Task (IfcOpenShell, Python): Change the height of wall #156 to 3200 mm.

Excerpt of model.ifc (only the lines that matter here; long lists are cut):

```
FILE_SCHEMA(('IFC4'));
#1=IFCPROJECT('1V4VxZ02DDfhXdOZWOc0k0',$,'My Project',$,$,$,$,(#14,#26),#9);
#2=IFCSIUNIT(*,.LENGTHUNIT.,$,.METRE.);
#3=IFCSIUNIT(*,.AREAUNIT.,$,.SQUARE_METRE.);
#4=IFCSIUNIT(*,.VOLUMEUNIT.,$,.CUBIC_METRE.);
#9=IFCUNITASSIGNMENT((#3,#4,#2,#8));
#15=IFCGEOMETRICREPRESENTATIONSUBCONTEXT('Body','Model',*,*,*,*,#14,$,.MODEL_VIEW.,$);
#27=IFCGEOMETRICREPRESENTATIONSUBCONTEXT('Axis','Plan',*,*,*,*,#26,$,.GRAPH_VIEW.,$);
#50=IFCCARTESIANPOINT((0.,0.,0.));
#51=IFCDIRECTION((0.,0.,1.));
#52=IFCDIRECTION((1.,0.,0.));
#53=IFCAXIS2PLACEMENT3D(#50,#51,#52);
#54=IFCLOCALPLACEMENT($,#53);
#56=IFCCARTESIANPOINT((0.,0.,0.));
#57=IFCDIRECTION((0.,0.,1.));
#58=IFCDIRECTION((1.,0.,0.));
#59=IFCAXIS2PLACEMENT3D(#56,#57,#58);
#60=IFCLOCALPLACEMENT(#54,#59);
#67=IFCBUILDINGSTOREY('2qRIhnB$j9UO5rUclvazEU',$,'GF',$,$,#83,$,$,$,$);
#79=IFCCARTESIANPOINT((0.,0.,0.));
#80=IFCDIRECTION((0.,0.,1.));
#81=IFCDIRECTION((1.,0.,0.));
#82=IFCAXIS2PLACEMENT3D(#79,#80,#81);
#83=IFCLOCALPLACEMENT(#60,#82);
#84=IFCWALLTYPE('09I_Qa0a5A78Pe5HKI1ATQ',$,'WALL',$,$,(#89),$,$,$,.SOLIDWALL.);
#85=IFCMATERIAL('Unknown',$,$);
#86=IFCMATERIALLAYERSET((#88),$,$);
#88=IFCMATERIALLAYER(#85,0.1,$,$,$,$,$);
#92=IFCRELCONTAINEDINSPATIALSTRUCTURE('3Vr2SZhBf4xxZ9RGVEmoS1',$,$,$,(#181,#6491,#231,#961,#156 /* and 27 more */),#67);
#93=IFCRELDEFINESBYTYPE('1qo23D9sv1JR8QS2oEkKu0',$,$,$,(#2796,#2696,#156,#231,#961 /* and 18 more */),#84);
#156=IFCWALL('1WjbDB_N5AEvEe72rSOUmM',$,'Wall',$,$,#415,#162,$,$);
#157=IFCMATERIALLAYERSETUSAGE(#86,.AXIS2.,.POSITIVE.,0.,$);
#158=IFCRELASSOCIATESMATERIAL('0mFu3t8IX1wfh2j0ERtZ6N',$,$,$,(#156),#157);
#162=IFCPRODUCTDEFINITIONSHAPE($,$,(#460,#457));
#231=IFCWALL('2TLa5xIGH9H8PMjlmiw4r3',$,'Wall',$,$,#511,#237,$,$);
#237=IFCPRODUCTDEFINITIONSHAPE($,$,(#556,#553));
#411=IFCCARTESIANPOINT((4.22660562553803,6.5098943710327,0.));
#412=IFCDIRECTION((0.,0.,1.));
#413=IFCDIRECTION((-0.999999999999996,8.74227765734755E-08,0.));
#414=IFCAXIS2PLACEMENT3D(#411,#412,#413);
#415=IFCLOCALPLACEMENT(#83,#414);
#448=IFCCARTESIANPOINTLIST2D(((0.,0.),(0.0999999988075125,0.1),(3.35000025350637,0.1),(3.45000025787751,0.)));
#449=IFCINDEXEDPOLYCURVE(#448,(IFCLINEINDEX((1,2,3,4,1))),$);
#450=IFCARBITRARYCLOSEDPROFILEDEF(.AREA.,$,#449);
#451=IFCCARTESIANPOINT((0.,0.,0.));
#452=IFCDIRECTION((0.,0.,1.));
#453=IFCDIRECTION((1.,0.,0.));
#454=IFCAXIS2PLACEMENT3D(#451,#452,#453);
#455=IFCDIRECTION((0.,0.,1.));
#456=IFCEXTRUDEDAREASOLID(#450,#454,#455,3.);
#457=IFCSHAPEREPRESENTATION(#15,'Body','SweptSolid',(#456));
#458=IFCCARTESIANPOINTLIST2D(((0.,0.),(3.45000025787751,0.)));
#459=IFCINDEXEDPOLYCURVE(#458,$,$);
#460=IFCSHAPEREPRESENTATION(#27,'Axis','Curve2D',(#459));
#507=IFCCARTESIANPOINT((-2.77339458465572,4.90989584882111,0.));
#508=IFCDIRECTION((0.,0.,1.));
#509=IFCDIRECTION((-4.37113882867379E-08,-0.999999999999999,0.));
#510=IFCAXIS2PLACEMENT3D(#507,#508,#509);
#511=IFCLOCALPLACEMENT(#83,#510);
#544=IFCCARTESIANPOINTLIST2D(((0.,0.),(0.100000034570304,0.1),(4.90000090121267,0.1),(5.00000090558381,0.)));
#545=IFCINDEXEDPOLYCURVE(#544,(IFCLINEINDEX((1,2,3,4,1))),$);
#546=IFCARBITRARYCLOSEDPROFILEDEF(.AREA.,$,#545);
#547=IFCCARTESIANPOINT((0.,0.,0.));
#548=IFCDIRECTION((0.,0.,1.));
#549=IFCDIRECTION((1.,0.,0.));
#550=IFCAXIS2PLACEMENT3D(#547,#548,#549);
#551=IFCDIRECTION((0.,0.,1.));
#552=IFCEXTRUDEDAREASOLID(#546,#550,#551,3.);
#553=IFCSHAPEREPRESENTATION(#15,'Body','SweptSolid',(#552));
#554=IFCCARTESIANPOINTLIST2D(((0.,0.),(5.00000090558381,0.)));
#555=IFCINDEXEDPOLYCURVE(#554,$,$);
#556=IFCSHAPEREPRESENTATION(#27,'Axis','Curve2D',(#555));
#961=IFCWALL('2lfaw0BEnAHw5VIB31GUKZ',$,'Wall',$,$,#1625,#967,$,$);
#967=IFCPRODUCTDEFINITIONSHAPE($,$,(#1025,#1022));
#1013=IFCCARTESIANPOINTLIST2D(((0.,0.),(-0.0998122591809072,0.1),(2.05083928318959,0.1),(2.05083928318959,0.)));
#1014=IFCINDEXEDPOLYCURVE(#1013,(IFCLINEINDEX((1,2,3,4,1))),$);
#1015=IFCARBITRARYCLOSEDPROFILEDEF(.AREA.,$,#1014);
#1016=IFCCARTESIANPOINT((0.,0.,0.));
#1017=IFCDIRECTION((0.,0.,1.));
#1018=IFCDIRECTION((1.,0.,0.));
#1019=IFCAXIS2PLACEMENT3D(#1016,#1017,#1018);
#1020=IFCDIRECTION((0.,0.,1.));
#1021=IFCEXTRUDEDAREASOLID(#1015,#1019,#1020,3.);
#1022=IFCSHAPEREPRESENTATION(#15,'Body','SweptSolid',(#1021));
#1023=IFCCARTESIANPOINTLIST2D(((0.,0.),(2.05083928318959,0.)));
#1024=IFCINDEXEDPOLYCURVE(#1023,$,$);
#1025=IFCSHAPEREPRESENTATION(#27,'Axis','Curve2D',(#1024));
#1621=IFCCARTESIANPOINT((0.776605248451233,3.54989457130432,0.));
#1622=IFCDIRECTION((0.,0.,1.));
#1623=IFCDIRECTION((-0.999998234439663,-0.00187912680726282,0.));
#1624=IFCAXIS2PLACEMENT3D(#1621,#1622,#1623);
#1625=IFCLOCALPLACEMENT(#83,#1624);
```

```python
import ifcopenshell
import ifcopenshell.geom
import ifcopenshell.util.representation
import ifcopenshell.util.shape
import ifcopenshell.util.unit

model = ifcopenshell.open("model.ifc")
unit_scale = ifcopenshell.util.unit.calculate_unit_scale(model)
settings = ifcopenshell.geom.settings()


def volume(element):
    """Net volume in cubic metres, openings subtracted."""
    shape = ifcopenshell.geom.create_shape(settings, element)
    return ifcopenshell.util.shape.get_volume(shape.geometry)


wall = model.by_guid("1WjbDB_N5AEvEe72rSOUmM")
before = volume(wall)

body = ifcopenshell.util.representation.get_representation(wall, "Model", "Body")
solid = body.Items[0]
old_height = solid.Depth
solid.Depth = 3.2 / unit_scale
after = volume(wall)

print(f"height {old_height:g} -> {solid.Depth:g}, volume {before:.3f} -> {after:.3f} m3")

model.write("model_updated.ifc")
```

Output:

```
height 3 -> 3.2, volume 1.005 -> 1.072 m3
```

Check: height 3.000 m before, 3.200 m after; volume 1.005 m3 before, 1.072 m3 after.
